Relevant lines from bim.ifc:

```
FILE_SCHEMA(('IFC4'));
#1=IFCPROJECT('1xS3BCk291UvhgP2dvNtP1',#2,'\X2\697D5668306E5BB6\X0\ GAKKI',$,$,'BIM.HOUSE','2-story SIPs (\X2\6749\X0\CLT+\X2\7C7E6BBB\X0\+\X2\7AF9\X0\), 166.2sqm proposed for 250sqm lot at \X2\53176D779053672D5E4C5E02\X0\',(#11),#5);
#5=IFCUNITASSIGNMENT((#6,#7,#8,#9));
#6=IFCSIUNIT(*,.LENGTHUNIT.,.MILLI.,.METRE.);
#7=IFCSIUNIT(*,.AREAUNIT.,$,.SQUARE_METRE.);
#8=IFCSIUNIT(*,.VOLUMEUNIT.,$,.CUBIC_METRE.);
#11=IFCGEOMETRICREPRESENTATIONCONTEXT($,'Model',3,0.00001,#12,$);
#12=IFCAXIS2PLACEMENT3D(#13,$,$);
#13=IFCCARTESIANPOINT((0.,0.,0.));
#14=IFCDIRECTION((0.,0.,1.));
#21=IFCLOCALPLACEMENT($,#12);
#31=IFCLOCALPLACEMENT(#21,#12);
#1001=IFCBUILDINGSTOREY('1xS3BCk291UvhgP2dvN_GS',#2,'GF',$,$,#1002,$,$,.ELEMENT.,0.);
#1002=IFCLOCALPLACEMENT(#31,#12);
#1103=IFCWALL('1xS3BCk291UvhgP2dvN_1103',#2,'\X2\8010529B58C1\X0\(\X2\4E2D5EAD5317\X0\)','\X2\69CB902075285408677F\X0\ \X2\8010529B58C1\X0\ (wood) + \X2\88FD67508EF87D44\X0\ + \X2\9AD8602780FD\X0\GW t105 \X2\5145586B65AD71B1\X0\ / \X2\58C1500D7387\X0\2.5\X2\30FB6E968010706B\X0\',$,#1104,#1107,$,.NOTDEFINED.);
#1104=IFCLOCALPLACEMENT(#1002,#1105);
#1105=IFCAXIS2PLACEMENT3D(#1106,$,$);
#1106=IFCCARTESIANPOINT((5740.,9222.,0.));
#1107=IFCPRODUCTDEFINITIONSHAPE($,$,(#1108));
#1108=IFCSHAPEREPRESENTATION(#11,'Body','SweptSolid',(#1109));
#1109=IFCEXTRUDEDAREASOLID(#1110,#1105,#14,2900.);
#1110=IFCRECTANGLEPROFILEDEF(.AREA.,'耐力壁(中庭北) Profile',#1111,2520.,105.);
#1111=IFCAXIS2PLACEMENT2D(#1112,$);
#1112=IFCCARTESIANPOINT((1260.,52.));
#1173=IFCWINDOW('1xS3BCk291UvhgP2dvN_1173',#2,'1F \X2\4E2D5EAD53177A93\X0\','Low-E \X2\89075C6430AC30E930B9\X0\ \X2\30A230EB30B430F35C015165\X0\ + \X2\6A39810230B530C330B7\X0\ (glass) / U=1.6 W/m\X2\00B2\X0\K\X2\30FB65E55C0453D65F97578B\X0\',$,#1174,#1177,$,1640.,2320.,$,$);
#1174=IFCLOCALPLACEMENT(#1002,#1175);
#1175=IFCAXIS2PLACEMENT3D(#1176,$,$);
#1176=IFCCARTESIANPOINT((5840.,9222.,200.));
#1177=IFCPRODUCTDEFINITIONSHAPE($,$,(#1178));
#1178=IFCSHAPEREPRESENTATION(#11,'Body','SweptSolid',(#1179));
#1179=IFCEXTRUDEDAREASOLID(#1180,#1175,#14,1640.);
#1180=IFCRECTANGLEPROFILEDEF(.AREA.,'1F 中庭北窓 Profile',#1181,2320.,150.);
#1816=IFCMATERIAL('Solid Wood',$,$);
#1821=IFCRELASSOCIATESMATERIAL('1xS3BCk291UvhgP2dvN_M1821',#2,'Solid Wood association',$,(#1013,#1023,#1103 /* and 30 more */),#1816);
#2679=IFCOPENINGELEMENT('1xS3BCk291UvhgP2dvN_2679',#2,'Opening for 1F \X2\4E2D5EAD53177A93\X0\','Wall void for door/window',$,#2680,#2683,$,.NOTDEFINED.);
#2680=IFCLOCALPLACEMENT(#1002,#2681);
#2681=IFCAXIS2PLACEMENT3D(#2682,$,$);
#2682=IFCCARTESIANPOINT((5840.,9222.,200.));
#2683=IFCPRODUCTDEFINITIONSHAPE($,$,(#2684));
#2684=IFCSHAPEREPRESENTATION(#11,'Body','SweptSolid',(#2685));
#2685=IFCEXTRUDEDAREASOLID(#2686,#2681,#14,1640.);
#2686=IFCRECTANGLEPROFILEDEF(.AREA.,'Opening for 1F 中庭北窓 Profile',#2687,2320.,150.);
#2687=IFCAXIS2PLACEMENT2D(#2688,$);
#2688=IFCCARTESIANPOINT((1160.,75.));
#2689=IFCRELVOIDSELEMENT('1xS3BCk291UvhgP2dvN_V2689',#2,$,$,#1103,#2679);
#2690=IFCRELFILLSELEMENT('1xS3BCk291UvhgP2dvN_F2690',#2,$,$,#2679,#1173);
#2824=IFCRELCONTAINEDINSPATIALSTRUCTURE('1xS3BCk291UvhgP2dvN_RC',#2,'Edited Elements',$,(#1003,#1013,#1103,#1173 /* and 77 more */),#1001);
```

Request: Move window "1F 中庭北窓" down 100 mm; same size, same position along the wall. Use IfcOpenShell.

```python
import numpy as np
import ifcopenshell
import ifcopenshell.api.geometry
import ifcopenshell.util.placement
import ifcopenshell.util.unit

model = ifcopenshell.open("bim.ifc")
unit_scale = ifcopenshell.util.unit.calculate_unit_scale(model)

window = model.by_id(1173)
opening = window.FillsVoids[0].RelatingOpeningElement
dz = -100.0

shift = np.array([0.0, 0.0, dz])
# The window is not placed relative to its opening, so move both.
for product in (opening, window):
    matrix = ifcopenshell.util.placement.get_local_placement(product.ObjectPlacement)
    matrix[:3, 3] += shift
    ifcopenshell.api.geometry.edit_object_placement(model, product=product, matrix=matrix, is_si=False)

print(f"moved by {dz * unit_scale:+.3f} m")

model.write("bim-out.ifc")
```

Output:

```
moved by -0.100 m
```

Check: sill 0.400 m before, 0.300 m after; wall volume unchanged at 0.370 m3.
